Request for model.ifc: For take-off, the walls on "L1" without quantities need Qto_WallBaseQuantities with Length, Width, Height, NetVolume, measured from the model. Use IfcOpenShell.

First a look at what the model holds.

```python
import ifcopenshell
import ifcopenshell.util.element
import ifcopenshell.util.unit

model = ifcopenshell.open("model.ifc")
print(model.schema)
for unit_type in ("LENGTHUNIT", "AREAUNIT", "VOLUMEUNIT"):
    print(unit_type, ifcopenshell.util.unit.calculate_unit_scale(model, unit_type))
storey = next(s for s in model.by_type("IfcBuildingStorey") if s.Name == "L1")
walls = [e for e in ifcopenshell.util.element.get_decomposition(storey) if e.is_a("IfcWall")]
for e in sorted(walls, key=lambda e: e.id()):
    print(e.id(), e.is_a(), e.Name, list(ifcopenshell.util.element.get_psets(e, qtos_only=True)), sep=" | ")
```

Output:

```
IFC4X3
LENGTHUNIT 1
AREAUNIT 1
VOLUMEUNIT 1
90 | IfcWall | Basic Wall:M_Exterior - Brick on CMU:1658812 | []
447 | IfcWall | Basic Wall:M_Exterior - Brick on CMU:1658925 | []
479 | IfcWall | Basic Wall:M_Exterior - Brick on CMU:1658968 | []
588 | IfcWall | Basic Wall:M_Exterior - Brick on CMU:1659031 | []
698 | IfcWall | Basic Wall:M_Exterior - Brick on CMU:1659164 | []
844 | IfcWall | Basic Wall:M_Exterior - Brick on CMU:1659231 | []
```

```python
import ifcopenshell
import ifcopenshell.api.pset
import ifcopenshell.geom
import ifcopenshell.util.element
import ifcopenshell.util.shape
import ifcopenshell.util.unit

model = ifcopenshell.open("model.ifc")
unit_scale = ifcopenshell.util.unit.calculate_unit_scale(model)
volume_scale = ifcopenshell.util.unit.calculate_unit_scale(model, "VOLUMEUNIT")
settings = ifcopenshell.geom.settings()

storey = next(s for s in model.by_type("IfcBuildingStorey") if s.Name == "L1")
walls = [e for e in ifcopenshell.util.element.get_decomposition(storey) if e.is_a("IfcWall")]

for e in sorted(walls, key=lambda e: e.id()):
    if ifcopenshell.util.element.get_psets(e, qtos_only=True, should_inherit=False):
        continue
    # Geometry comes back in metres, in the element's own axes.
    shape = ifcopenshell.geom.create_shape(settings, e)
    values = {
        "Length": ifcopenshell.util.shape.get_x(shape.geometry) / unit_scale,
        "Width": ifcopenshell.util.shape.get_y(shape.geometry) / unit_scale,
        "Height": ifcopenshell.util.shape.get_z(shape.geometry) / unit_scale,
        "NetVolume": ifcopenshell.util.shape.get_volume(shape.geometry) / volume_scale,
    }
    qto = ifcopenshell.api.pset.add_qto(model, product=e, name="Qto_WallBaseQuantities")
    ifcopenshell.api.pset.edit_qto(model, qto=qto, properties=values)
    print(e.id(), {k: round(v, 3) for k, v in values.items()})

model.write("model_edited.ifc")
```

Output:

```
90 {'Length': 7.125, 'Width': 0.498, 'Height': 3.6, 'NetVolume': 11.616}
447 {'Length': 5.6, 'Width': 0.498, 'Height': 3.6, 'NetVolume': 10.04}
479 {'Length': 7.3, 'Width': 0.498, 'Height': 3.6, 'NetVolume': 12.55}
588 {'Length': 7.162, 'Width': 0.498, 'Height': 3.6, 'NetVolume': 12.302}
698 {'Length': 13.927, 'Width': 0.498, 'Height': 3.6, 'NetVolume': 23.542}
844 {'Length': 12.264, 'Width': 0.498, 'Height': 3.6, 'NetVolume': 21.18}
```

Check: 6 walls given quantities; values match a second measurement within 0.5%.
